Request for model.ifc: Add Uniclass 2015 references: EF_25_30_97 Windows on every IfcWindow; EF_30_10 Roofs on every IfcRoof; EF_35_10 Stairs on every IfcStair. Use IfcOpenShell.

First a look at what the model holds.

```python
import ifcopenshell

model = ifcopenshell.open("model.ifc")
print(model.schema)
print("classifications:", [c.Name for c in model.by_type("IfcClassification")])
for ifc_class in ("IfcDoor", "IfcRoof", "IfcStair", "IfcWall", "IfcWindow"):
    print(ifc_class, len(model.by_type(ifc_class)))
```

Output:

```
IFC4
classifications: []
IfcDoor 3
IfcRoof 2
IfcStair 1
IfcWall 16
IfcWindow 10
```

```python
import ifcopenshell
import ifcopenshell.api.classification

model = ifcopenshell.open("model.ifc")

system = ifcopenshell.api.classification.add_classification(model, classification="Uniclass 2015")

codes = {
    "IfcWindow": ("EF_25_30_97", "Windows"),
    "IfcRoof": ("EF_30_10", "Roofs"),
    "IfcStair": ("EF_35_10", "Stairs"),
}
for ifc_class, (code, name) in codes.items():
    products = model.by_type(ifc_class)
    ifcopenshell.api.classification.add_reference(
        model, products=products, classification=system, identification=code, name=name
    )
    print(code, len(products))

model.write("model_edited.ifc")
```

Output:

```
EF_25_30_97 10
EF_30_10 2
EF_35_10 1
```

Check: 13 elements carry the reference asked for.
